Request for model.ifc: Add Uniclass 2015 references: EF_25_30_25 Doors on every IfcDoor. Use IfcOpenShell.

First a look at what the model holds.

```python
import ifcopenshell

model = ifcopenshell.open("model.ifc")
print(model.schema)
print("classifications:", [c.Name for c in model.by_type("IfcClassification")])
for ifc_class in ("IfcDoor", "IfcRoof", "IfcStair", "IfcWall", "IfcWindow"):
    print(ifc_class, len(model.by_type(ifc_class)))
```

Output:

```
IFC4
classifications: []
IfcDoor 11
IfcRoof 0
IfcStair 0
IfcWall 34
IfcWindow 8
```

```python
import ifcopenshell
import ifcopenshell.api.classification

model = ifcopenshell.open("model.ifc")

system = ifcopenshell.api.classification.add_classification(model, classification="Uniclass 2015")

codes = {
    "IfcDoor": ("EF_25_30_25", "Doors"),
}
for ifc_class, (code, name) in codes.items():
    products = model.by_type(ifc_class)
    ifcopenshell.api.classification.add_reference(
        model, products=products, classification=system, identification=code, name=name
    )
    print(code, len(products))

model.write("model_updated.ifc")
```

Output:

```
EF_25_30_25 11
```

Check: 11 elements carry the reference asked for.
